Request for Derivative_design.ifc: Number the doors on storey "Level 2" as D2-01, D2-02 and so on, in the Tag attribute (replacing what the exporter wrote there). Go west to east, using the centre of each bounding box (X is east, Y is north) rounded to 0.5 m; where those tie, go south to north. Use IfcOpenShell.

First a look at what the model holds.

```python
import ifcopenshell
import ifcopenshell.util.element
import ifcopenshell.util.placement

model = ifcopenshell.open("Derivative_design.ifc")
print(model.schema)
storey = next(s for s in model.by_type("IfcBuildingStorey") if s.Name == "Level 2")
doors = [e for e in ifcopenshell.util.element.get_decomposition(storey) if e.is_a("IfcDoor")]
for e in sorted(doors, key=lambda e: e.id()):
    origin = ifcopenshell.util.placement.get_local_placement(e.ObjectPlacement)[:3, 3]
    print(e.id(), e.Tag, e.Name, origin.round(2) + 0.0, sep=" | ")
```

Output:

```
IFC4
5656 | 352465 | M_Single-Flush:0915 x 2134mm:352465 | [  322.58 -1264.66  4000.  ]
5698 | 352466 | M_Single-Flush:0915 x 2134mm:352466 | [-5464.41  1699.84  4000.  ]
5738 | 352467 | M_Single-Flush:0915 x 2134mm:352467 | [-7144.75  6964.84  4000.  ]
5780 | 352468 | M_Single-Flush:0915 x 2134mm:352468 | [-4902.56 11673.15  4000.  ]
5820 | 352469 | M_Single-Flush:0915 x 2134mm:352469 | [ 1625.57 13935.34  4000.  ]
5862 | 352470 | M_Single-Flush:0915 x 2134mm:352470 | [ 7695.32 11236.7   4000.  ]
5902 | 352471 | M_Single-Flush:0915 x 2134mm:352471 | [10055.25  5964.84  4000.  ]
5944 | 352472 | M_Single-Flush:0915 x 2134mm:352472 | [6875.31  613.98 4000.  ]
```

```python
import ifcopenshell
import ifcopenshell.geom
import ifcopenshell.util.element
import ifcopenshell.util.shape

model = ifcopenshell.open("Derivative_design.ifc")
settings = ifcopenshell.geom.settings()
settings.set("use-world-coords", True)


def centre(element):
    shape = ifcopenshell.geom.create_shape(settings, element)
    return ifcopenshell.util.shape.get_bbox_centroid(shape.geometry)


storey = next(s for s in model.by_type("IfcBuildingStorey") if s.Name == "Level 2")
doors = [e for e in ifcopenshell.util.element.get_decomposition(storey) if e.is_a("IfcDoor")]

# Insertion points can sit at a corner or the storey origin, so sort by the geometry (in metres).
centres = {e: centre(e) for e in doors}
doors.sort(key=lambda e: (round(centres[e][0] / 0.5), centres[e][1]))

for i, e in enumerate(doors, start=1):
    number = f"D2-{i:02d}"
    e.Tag = number
    print(e.id(), number)

model.write("Derivative_design_edited.ifc")
```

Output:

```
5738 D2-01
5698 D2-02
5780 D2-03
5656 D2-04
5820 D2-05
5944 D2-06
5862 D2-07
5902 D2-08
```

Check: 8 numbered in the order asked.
